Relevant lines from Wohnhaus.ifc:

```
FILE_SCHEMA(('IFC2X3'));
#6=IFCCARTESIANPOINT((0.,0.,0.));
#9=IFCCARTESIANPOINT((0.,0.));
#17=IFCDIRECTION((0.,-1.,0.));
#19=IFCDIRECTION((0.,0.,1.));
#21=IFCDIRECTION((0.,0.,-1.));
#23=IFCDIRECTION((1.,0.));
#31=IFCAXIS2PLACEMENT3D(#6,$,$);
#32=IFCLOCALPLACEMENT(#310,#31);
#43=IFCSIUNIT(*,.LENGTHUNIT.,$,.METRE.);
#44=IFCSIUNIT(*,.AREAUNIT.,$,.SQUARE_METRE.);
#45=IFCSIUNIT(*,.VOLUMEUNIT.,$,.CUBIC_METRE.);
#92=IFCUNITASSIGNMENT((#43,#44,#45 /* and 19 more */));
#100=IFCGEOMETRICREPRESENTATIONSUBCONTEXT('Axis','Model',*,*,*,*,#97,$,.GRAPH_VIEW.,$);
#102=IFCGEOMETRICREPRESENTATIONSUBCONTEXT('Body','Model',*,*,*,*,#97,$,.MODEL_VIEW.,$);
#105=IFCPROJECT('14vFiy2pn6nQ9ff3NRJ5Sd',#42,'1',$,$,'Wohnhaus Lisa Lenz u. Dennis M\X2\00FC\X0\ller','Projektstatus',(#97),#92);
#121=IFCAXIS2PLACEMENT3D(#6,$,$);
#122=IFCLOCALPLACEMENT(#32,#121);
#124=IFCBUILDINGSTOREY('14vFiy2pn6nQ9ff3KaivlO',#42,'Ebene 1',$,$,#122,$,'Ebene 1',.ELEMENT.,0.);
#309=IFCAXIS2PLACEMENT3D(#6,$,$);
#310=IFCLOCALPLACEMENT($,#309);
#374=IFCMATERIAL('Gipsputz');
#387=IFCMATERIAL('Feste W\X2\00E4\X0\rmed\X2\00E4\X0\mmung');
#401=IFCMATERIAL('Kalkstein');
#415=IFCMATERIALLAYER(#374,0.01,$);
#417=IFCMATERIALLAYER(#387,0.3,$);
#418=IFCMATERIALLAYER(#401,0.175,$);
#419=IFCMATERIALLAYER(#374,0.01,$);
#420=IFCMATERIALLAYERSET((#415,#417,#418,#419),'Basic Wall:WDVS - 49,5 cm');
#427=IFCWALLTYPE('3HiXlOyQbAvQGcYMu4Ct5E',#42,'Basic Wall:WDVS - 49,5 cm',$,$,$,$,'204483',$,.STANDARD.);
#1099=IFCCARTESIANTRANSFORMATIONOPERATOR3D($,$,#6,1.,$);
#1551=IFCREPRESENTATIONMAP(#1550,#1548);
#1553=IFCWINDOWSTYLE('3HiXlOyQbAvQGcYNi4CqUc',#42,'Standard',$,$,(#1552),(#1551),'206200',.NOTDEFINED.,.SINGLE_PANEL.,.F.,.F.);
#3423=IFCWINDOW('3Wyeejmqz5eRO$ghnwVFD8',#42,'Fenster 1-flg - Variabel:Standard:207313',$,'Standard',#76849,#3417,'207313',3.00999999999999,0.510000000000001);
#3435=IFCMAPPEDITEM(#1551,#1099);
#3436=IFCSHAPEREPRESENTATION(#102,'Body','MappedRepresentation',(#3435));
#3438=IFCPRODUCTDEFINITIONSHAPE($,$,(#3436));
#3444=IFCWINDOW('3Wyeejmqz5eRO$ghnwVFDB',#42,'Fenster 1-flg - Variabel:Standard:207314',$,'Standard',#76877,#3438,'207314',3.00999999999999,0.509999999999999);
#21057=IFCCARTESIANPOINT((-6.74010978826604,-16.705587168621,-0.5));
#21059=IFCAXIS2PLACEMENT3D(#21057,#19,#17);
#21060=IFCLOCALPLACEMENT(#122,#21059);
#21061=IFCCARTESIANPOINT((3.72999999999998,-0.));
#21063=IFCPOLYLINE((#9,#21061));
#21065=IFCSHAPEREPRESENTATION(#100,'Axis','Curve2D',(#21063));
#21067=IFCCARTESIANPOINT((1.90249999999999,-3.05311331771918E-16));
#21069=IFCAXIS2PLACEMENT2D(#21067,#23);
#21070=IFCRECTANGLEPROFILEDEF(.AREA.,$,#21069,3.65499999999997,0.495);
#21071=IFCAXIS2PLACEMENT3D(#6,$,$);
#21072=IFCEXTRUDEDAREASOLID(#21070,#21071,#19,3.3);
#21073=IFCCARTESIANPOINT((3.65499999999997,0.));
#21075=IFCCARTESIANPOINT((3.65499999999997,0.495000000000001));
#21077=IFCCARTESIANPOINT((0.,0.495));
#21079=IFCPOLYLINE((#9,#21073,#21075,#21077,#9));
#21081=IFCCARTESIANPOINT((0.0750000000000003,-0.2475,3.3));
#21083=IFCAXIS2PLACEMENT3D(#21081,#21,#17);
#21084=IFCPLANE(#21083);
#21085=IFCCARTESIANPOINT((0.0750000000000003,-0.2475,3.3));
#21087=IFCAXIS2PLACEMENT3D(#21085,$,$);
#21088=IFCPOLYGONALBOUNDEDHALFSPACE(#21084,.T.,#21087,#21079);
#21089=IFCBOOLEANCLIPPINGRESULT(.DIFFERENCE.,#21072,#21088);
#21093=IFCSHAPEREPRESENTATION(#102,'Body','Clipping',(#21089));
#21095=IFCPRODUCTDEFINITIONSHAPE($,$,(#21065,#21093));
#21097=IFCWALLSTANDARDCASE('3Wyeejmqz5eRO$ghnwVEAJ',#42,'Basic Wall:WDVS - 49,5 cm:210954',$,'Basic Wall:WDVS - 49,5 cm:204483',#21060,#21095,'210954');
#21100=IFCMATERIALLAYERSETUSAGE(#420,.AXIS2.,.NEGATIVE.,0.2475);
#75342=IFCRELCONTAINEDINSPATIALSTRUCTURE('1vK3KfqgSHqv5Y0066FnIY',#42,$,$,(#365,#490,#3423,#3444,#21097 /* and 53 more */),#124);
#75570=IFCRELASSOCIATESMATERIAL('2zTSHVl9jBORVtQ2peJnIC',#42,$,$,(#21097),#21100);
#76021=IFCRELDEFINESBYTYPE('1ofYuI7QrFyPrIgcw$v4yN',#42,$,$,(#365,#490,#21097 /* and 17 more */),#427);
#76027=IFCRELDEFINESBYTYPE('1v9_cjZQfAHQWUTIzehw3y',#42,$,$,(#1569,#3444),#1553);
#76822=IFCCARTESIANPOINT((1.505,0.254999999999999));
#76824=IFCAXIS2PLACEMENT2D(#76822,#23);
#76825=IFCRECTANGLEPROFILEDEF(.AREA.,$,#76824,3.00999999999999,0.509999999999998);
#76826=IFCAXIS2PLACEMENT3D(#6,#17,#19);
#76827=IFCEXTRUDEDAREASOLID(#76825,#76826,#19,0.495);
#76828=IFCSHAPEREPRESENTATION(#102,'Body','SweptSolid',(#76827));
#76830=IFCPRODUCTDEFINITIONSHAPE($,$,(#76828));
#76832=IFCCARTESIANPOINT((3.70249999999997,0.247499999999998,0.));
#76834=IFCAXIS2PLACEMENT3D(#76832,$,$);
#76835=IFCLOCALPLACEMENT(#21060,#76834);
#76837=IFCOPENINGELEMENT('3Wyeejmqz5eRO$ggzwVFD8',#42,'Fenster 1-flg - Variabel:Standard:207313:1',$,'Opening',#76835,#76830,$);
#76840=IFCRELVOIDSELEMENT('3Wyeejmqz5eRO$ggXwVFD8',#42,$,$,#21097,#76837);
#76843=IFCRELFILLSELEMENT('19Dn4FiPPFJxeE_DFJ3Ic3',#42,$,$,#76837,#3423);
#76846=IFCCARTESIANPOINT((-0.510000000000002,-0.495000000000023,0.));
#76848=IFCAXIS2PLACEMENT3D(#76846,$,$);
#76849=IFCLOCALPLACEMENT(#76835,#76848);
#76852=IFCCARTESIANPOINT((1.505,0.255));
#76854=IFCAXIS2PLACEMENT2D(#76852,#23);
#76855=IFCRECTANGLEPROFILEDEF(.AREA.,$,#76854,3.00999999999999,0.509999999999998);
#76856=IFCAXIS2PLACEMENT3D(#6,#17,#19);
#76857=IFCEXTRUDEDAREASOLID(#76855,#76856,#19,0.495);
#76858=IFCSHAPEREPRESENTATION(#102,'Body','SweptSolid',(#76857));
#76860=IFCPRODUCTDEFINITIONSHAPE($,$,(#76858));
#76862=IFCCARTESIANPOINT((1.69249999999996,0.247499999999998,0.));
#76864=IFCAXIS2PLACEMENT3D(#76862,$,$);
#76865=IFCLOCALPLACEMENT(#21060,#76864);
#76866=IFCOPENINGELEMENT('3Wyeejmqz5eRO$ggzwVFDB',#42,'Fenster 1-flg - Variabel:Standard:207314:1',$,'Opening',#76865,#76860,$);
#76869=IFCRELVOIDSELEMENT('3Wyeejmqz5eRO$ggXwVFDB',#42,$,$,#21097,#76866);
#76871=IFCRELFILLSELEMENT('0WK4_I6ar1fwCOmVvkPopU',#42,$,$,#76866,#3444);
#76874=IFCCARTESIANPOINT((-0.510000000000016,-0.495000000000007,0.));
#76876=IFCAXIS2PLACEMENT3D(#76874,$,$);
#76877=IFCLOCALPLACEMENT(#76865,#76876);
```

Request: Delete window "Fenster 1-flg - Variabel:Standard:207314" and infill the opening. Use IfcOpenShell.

```python
import ifcopenshell
import ifcopenshell.api.feature
import ifcopenshell.api.root
import ifcopenshell.geom
import ifcopenshell.util.shape

model = ifcopenshell.open("Wohnhaus.ifc")
settings = ifcopenshell.geom.settings()


def volume(element):
    """Net volume in cubic metres, openings subtracted."""
    shape = ifcopenshell.geom.create_shape(settings, element)
    return ifcopenshell.util.shape.get_volume(shape.geometry)


window = model.by_guid("3Wyeejmqz5eRO$ghnwVFDB")
opening = window.FillsVoids[0].RelatingOpeningElement
wall = opening.VoidsElements[0].RelatingBuildingElement
before = volume(wall)

ifcopenshell.api.root.remove_product(model, product=window)
ifcopenshell.api.feature.remove_feature(model, feature=opening)

after = volume(wall)

print(f"wall volume {before:.3f} -> {after:.3f} m3")

model.write("Wohnhaus_edited.ifc")
```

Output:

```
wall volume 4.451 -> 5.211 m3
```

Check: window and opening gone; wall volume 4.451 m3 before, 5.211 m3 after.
